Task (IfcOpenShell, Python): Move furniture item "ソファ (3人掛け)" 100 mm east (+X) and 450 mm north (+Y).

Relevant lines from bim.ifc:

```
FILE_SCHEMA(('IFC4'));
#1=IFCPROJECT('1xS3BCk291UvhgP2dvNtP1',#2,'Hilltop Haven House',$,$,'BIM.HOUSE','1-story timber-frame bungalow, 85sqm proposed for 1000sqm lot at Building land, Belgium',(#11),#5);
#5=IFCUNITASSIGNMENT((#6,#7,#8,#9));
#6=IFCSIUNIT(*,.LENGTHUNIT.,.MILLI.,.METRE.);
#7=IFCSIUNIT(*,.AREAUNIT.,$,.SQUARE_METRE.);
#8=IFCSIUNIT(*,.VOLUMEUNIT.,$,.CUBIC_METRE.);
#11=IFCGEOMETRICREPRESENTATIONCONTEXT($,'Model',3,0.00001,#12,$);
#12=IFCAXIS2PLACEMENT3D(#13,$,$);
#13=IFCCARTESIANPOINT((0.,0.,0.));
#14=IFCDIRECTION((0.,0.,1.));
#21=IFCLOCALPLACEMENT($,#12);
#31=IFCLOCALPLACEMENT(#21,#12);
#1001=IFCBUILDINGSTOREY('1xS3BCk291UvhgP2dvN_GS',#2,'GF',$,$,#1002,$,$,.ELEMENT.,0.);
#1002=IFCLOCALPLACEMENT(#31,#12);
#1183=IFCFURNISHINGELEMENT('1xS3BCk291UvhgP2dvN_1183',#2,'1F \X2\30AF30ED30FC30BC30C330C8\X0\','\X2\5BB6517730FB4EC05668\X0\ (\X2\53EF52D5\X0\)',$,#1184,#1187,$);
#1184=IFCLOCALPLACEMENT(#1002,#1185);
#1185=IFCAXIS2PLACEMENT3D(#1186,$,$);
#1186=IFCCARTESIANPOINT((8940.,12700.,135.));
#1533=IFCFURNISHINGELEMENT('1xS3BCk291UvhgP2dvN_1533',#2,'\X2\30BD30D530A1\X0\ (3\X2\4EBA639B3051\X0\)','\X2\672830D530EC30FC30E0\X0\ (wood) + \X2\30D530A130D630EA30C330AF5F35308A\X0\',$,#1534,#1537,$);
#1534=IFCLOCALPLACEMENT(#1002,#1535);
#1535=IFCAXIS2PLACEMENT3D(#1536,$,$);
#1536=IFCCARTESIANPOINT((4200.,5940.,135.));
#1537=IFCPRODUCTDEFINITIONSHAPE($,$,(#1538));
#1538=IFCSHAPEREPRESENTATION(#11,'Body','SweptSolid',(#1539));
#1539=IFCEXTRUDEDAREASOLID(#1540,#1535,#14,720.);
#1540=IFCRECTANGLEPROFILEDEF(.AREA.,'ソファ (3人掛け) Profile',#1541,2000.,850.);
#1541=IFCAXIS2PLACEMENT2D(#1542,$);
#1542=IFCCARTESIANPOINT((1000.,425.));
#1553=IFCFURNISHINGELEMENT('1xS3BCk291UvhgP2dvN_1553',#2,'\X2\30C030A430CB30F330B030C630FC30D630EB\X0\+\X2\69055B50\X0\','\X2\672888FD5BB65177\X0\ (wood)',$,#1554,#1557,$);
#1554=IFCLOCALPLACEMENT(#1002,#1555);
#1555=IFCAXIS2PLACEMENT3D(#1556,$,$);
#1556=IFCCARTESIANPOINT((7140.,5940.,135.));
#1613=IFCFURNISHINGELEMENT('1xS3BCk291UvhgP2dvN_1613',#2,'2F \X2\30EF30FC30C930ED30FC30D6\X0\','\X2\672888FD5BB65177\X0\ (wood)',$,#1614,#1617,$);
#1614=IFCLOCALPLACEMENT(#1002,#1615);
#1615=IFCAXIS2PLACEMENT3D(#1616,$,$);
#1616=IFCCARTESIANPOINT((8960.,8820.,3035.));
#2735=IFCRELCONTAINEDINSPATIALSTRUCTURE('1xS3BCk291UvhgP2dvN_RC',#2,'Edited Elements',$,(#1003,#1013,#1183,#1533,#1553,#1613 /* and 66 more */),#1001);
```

```python
import ifcopenshell
import ifcopenshell.api.geometry
import ifcopenshell.util.placement
import ifcopenshell.util.unit

model = ifcopenshell.open("bim.ifc")
unit_scale = ifcopenshell.util.unit.calculate_unit_scale(model)

item = model.by_id(1533)
matrix = ifcopenshell.util.placement.get_local_placement(item.ObjectPlacement)
matrix[0, 3] += 0.1 / unit_scale
matrix[1, 3] += 0.45 / unit_scale
ifcopenshell.api.geometry.edit_object_placement(model, product=item, matrix=matrix, is_si=False)

print(ifcopenshell.util.placement.get_local_placement(item.ObjectPlacement).round(3) + 0.0)

model.write("bim_edited.ifc")
```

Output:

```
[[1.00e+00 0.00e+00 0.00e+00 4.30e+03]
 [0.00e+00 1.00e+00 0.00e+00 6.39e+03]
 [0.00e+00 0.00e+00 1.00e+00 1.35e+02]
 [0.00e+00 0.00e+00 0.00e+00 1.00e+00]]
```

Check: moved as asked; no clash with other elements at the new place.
